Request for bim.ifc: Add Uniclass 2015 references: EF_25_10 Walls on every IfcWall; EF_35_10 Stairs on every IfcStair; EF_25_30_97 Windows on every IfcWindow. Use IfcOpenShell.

First a look at what the model holds.

```python
import ifcopenshell

model = ifcopenshell.open("bim.ifc")
print(model.schema)
print("classifications:", [c.Name for c in model.by_type("IfcClassification")])
for ifc_class in ("IfcDoor", "IfcRoof", "IfcStair", "IfcWall", "IfcWindow"):
    print(ifc_class, len(model.by_type(ifc_class)))
```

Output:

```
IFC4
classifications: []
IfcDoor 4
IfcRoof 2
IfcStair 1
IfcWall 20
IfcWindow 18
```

```python
import ifcopenshell
import ifcopenshell.api.classification

model = ifcopenshell.open("bim.ifc")

system = ifcopenshell.api.classification.add_classification(model, classification="Uniclass 2015")

codes = {
    "IfcWall": ("EF_25_10", "Walls"),
    "IfcStair": ("EF_35_10", "Stairs"),
    "IfcWindow": ("EF_25_30_97", "Windows"),
}
for ifc_class, (code, name) in codes.items():
    products = model.by_type(ifc_class)
    ifcopenshell.api.classification.add_reference(
        model, products=products, classification=system, identification=code, name=name
    )
    print(code, len(products))

model.write("bim_rev.ifc")
```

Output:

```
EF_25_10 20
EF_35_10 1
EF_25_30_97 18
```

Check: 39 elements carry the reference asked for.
